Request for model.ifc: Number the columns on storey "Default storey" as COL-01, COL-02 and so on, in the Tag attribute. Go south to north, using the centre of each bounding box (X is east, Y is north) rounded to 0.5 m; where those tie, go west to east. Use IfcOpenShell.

First a look at what the model holds.

```python
import ifcopenshell
import ifcopenshell.util.element
import ifcopenshell.util.placement

model = ifcopenshell.open("model.ifc")
print(model.schema)
storey = next(s for s in model.by_type("IfcBuildingStorey") if s.Name == "Default storey")
columns = [e for e in ifcopenshell.util.element.get_decomposition(storey) if e.is_a("IfcColumn")]
for e in sorted(columns, key=lambda e: e.id()):
    origin = ifcopenshell.util.placement.get_local_placement(e.ObjectPlacement)[:3, 3]
    print(e.id(), e.Tag, e.Name, origin.round(2) + 0.0, sep=" | ")
```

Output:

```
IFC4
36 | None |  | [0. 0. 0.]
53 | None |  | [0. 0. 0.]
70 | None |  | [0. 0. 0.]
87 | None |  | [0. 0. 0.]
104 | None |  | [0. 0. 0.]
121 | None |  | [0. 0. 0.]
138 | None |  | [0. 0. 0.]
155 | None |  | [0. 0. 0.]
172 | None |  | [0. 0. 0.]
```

```python
import ifcopenshell
import ifcopenshell.geom
import ifcopenshell.util.element
import ifcopenshell.util.shape

model = ifcopenshell.open("model.ifc")
settings = ifcopenshell.geom.settings()
settings.set("use-world-coords", True)


def centre(element):
    shape = ifcopenshell.geom.create_shape(settings, element)
    return ifcopenshell.util.shape.get_bbox_centroid(shape.geometry)


storey = next(s for s in model.by_type("IfcBuildingStorey") if s.Name == "Default storey")
columns = [e for e in ifcopenshell.util.element.get_decomposition(storey) if e.is_a("IfcColumn")]

# Insertion points can sit at a corner or the storey origin, so sort by the geometry (in metres).
centres = {e: centre(e) for e in columns}
columns.sort(key=lambda e: (round(centres[e][1] / 0.5), centres[e][0]))

for i, e in enumerate(columns, start=1):
    number = f"COL-{i:02d}"
    e.Tag = number
    print(e.id(), number)

model.write("model_edited.ifc")
```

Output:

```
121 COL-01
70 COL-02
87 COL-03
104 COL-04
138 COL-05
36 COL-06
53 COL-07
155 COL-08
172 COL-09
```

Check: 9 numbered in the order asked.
